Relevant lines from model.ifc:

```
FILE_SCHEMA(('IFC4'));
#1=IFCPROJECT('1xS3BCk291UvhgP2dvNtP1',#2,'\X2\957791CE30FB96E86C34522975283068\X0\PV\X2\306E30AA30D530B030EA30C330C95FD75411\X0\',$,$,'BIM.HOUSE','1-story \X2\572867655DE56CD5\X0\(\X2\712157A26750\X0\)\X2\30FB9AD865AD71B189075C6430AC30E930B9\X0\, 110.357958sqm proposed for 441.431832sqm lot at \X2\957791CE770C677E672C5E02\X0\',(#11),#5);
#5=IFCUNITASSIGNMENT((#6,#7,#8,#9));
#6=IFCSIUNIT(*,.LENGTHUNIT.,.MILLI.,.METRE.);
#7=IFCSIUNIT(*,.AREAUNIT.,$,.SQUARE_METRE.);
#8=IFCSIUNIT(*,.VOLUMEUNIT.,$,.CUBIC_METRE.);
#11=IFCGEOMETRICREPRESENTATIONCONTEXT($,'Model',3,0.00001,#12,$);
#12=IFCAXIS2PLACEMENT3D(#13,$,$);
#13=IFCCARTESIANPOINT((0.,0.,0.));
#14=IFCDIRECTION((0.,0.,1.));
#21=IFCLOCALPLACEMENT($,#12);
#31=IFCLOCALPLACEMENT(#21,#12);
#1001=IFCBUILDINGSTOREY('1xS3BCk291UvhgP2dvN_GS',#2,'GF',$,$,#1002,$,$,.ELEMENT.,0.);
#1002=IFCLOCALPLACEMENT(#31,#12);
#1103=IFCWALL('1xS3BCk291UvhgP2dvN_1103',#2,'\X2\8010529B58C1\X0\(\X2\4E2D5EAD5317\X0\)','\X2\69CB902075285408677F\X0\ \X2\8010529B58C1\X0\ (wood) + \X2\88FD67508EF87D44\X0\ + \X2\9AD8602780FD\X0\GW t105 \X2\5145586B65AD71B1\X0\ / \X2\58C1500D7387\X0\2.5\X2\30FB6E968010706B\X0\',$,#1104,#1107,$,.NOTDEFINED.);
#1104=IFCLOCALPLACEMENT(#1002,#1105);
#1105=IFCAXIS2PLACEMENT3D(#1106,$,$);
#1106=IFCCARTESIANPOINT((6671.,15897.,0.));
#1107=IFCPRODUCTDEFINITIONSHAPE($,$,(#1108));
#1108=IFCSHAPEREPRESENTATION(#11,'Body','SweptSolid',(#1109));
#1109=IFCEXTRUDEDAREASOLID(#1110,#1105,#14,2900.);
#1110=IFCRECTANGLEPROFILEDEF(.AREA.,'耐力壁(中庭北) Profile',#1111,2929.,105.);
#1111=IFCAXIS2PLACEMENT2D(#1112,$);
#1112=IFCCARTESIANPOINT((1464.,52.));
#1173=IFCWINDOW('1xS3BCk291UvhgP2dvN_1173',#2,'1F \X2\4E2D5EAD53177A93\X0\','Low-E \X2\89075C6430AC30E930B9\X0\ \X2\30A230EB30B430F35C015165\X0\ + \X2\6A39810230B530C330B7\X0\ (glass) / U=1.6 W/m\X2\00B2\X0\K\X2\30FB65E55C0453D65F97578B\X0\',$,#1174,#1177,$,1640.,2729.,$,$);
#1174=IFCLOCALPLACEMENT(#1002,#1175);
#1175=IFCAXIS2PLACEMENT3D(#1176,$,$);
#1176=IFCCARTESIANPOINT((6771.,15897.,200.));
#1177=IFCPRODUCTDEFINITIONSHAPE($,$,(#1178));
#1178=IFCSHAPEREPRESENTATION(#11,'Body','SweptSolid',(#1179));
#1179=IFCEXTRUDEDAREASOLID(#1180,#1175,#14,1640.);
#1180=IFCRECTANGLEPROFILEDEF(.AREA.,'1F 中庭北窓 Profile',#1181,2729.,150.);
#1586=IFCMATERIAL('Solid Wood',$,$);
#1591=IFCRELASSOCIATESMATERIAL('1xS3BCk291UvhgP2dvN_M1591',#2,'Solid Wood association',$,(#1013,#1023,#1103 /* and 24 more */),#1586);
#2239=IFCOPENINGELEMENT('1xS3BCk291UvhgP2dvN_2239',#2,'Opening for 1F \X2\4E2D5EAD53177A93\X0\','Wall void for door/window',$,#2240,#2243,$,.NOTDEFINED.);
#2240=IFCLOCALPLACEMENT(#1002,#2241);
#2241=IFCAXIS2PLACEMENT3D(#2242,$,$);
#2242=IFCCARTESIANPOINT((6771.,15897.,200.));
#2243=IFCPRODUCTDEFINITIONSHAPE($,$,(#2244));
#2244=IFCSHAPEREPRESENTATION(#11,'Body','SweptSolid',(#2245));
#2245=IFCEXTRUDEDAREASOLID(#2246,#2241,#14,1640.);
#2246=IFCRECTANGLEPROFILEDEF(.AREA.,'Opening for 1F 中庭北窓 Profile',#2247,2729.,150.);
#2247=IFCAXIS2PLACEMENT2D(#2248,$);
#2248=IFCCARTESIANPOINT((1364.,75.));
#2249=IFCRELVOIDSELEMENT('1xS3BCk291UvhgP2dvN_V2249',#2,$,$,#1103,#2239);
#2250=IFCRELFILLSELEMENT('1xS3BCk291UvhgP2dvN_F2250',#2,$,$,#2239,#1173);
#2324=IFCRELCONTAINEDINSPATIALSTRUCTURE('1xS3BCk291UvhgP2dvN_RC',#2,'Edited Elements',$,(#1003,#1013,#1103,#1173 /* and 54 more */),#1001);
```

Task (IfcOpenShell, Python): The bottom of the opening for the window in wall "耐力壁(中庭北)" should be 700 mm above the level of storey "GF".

```python
import numpy as np
import ifcopenshell
import ifcopenshell.api.geometry
import ifcopenshell.geom
import ifcopenshell.util.element
import ifcopenshell.util.placement
import ifcopenshell.util.shape
import ifcopenshell.util.unit

model = ifcopenshell.open("model.ifc")
unit_scale = ifcopenshell.util.unit.calculate_unit_scale(model)

window = model.by_id(1173)
opening = window.FillsVoids[0].RelatingOpeningElement
storey = ifcopenshell.util.element.get_container(window, ifc_class="IfcBuildingStorey")
level = ifcopenshell.util.placement.get_local_placement(storey.ObjectPlacement)[2, 3]

# The opening's origin need not be at the sill, so measure its lowest point.
shape = ifcopenshell.geom.create_shape(ifcopenshell.geom.settings(), opening)
bottom = ifcopenshell.util.shape.get_shape_bottom_elevation(shape, shape.geometry) / unit_scale
dz = level + 0.7 / unit_scale - bottom

shift = np.array([0.0, 0.0, dz])
# The window is not placed relative to its opening, so move both.
for product in (opening, window):
    matrix = ifcopenshell.util.placement.get_local_placement(product.ObjectPlacement)
    matrix[:3, 3] += shift
    ifcopenshell.api.geometry.edit_object_placement(model, product=product, matrix=matrix, is_si=False)

print(f"moved by {dz * unit_scale:+.3f} m")

model.write("model_edited.ifc")
```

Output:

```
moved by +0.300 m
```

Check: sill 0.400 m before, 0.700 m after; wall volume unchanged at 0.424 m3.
